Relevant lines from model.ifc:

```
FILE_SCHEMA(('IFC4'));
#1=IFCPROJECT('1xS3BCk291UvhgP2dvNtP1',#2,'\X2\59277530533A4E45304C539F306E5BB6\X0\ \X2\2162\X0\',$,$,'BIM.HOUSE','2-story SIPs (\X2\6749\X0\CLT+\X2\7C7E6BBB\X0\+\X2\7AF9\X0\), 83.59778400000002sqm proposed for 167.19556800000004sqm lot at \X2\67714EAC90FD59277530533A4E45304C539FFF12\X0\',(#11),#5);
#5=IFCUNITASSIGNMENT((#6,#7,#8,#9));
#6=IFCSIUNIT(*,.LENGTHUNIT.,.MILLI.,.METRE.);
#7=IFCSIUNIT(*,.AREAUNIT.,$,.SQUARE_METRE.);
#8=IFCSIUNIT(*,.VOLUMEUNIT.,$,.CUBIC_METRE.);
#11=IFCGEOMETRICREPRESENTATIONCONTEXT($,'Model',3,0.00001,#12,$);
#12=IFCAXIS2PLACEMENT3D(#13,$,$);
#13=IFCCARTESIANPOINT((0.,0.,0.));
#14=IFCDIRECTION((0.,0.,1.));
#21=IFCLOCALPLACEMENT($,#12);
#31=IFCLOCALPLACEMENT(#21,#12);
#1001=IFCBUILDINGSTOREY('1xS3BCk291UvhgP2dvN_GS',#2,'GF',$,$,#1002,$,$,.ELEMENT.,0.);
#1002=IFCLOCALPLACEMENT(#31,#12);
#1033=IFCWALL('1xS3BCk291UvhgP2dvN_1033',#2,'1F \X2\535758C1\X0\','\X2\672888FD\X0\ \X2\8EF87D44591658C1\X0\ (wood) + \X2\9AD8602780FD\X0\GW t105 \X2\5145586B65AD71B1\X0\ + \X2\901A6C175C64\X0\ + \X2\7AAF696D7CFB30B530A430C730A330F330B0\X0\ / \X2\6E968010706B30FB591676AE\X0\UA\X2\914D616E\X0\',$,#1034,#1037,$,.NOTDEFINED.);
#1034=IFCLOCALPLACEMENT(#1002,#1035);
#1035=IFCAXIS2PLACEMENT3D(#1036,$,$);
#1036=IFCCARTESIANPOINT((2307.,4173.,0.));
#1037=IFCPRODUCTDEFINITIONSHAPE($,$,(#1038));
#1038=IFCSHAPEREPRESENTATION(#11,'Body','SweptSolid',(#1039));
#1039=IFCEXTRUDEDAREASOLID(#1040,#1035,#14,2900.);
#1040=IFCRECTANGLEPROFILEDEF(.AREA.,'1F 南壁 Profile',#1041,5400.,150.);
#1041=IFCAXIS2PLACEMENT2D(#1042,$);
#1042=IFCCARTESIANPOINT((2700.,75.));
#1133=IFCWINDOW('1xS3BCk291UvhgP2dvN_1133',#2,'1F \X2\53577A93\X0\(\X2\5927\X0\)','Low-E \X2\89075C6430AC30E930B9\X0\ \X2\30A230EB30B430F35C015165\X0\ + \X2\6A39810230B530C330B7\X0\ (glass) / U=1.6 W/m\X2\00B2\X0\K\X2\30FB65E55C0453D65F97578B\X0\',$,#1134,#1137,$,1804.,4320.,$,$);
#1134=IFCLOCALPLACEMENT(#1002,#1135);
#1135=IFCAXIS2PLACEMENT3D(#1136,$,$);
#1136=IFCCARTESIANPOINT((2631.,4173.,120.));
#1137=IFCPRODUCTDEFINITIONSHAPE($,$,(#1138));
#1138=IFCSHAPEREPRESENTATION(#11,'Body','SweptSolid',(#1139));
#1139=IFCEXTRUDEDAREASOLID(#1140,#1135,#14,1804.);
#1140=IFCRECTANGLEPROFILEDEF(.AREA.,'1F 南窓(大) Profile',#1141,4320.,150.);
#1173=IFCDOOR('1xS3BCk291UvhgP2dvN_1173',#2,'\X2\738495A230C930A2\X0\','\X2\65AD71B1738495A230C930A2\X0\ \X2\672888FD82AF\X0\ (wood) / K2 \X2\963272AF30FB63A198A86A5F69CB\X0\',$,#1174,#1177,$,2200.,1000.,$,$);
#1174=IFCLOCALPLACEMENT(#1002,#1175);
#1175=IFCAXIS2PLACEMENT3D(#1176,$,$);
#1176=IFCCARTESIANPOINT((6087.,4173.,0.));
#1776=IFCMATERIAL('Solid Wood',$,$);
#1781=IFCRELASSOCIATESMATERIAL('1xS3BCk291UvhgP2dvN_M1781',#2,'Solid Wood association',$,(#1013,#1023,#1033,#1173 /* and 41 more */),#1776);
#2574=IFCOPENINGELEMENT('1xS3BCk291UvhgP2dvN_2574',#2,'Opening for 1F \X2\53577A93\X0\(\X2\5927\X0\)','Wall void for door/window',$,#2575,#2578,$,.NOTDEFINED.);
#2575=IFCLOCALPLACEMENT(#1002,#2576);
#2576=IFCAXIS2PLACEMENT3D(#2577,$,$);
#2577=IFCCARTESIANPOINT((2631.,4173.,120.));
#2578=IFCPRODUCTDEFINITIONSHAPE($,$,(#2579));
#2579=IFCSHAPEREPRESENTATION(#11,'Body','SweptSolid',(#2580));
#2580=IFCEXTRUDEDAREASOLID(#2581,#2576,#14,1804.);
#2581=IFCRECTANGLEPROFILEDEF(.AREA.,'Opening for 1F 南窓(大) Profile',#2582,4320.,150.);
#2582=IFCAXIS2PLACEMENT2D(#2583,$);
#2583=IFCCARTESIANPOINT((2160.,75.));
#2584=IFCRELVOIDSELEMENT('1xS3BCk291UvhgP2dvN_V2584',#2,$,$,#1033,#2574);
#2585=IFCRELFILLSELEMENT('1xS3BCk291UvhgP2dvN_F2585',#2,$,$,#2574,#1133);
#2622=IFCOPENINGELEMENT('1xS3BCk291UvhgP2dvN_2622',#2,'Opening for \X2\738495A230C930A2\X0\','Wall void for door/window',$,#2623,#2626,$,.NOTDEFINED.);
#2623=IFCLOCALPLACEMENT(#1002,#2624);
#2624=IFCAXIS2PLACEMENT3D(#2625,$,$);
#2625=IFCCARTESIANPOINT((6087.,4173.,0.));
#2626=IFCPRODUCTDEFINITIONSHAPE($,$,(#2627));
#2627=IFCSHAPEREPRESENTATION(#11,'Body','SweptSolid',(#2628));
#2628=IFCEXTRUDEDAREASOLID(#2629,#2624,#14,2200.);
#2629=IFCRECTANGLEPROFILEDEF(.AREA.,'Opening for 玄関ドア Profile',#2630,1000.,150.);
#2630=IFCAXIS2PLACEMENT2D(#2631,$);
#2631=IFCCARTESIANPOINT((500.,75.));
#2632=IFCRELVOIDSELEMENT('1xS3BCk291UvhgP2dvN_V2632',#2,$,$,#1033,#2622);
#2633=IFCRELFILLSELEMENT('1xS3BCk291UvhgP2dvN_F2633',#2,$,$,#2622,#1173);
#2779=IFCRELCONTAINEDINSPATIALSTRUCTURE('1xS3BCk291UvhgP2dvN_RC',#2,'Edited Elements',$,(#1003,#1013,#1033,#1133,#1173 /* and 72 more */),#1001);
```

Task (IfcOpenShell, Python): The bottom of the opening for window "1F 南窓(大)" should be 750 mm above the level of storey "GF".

```python
import numpy as np
import ifcopenshell
import ifcopenshell.api.geometry
import ifcopenshell.geom
import ifcopenshell.util.element
import ifcopenshell.util.placement
import ifcopenshell.util.shape
import ifcopenshell.util.unit

model = ifcopenshell.open("model.ifc")
unit_scale = ifcopenshell.util.unit.calculate_unit_scale(model)

window = model.by_guid("1xS3BCk291UvhgP2dvN_1133")
opening = window.FillsVoids[0].RelatingOpeningElement
storey = ifcopenshell.util.element.get_container(window, ifc_class="IfcBuildingStorey")
level = ifcopenshell.util.placement.get_local_placement(storey.ObjectPlacement)[2, 3]

# The opening's origin need not be at the sill, so measure its lowest point.
shape = ifcopenshell.geom.create_shape(ifcopenshell.geom.settings(), opening)
bottom = ifcopenshell.util.shape.get_shape_bottom_elevation(shape, shape.geometry) / unit_scale
dz = level + 750.0 - bottom

shift = np.array([0.0, 0.0, dz])
# The window is not placed relative to its opening, so move both.
for product in (opening, window):
    matrix = ifcopenshell.util.placement.get_local_placement(product.ObjectPlacement)
    matrix[:3, 3] += shift
    ifcopenshell.api.geometry.edit_object_placement(model, product=product, matrix=matrix, is_si=False)

print(f"moved by {dz * unit_scale:+.3f} m")

model.write("model_edited.ifc")
```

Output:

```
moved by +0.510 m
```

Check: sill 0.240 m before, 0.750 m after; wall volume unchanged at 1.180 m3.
